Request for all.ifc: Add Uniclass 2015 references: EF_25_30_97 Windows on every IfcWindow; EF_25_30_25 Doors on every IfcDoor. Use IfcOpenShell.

First a look at what the model holds.

```python
import ifcopenshell

model = ifcopenshell.open("all.ifc")
print(model.schema)
print("classifications:", [c.Name for c in model.by_type("IfcClassification")])
for ifc_class in ("IfcDoor", "IfcRoof", "IfcStair", "IfcWall", "IfcWindow"):
    print(ifc_class, len(model.by_type(ifc_class)))
```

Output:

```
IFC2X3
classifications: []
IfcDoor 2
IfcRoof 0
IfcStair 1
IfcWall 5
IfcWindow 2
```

```python
import ifcopenshell
import ifcopenshell.api.classification

model = ifcopenshell.open("all.ifc")

# IFC2X3 requires Source and Edition and has no link from the project to the system.
system = model.create_entity("IfcClassification", Source="NBS", Edition="2015", Name="Uniclass 2015")

codes = {
    "IfcWindow": ("EF_25_30_97", "Windows"),
    "IfcDoor": ("EF_25_30_25", "Doors"),
}
for ifc_class, (code, name) in codes.items():
    products = model.by_type(ifc_class)
    ifcopenshell.api.classification.add_reference(
        model, products=products, classification=system, identification=code, name=name
    )
    print(code, len(products))

model.write("all_v2.ifc")
```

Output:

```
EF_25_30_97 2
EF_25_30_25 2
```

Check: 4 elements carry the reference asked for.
